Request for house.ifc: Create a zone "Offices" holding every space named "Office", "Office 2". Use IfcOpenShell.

First a look at what the model holds.

```python
import ifcopenshell

model = ifcopenshell.open("house.ifc")
print(model.schema)
seen = {}
for space in model.by_type("IfcSpace"):
    seen[space.LongName] = seen.get(space.LongName, 0) + 1
for name, count in sorted(seen.items(), key=str):
    print(count, "x", name)
print("zones:", [z.Name for z in model.by_type("IfcZone")][:20])
```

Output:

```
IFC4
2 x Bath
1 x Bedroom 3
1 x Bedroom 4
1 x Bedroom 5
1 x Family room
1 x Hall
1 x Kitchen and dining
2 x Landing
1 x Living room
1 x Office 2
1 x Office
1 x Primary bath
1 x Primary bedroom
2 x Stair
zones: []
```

```python
import ifcopenshell
import ifcopenshell.api.group
import ifcopenshell.api.root

model = ifcopenshell.open("house.ifc")

names = {"Office", "Office 2"}
spaces = [s for s in model.by_type("IfcSpace") if s.LongName in names]

zone = ifcopenshell.api.root.create_entity(model, ifc_class="IfcZone", name="Offices")
ifcopenshell.api.group.assign_group(model, products=spaces, group=zone)
print(len(spaces), "spaces in", zone.Name)

model.write("house-out.ifc")
```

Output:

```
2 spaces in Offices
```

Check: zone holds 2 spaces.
